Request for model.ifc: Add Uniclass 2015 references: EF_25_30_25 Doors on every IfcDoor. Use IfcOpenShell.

First a look at what the model holds.

```python
import ifcopenshell

model = ifcopenshell.open("model.ifc")
print(model.schema)
print("classifications:", [c.Name for c in model.by_type("IfcClassification")])
for ifc_class in ("IfcDoor", "IfcRoof", "IfcStair", "IfcWall", "IfcWindow"):
    print(ifc_class, len(model.by_type(ifc_class)))
```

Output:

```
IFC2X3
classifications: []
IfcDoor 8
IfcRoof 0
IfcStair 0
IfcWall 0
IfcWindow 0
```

```python
import ifcopenshell
import ifcopenshell.api.classification

model = ifcopenshell.open("model.ifc")

# IFC2X3 requires Source and Edition and has no link from the project to the system.
system = model.create_entity("IfcClassification", Source="NBS", Edition="2015", Name="Uniclass 2015")

codes = {
    "IfcDoor": ("EF_25_30_25", "Doors"),
}
for ifc_class, (code, name) in codes.items():
    products = model.by_type(ifc_class)
    ifcopenshell.api.classification.add_reference(
        model, products=products, classification=system, identification=code, name=name
    )
    print(code, len(products))

model.write("model-out.ifc")
```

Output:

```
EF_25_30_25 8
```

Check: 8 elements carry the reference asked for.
